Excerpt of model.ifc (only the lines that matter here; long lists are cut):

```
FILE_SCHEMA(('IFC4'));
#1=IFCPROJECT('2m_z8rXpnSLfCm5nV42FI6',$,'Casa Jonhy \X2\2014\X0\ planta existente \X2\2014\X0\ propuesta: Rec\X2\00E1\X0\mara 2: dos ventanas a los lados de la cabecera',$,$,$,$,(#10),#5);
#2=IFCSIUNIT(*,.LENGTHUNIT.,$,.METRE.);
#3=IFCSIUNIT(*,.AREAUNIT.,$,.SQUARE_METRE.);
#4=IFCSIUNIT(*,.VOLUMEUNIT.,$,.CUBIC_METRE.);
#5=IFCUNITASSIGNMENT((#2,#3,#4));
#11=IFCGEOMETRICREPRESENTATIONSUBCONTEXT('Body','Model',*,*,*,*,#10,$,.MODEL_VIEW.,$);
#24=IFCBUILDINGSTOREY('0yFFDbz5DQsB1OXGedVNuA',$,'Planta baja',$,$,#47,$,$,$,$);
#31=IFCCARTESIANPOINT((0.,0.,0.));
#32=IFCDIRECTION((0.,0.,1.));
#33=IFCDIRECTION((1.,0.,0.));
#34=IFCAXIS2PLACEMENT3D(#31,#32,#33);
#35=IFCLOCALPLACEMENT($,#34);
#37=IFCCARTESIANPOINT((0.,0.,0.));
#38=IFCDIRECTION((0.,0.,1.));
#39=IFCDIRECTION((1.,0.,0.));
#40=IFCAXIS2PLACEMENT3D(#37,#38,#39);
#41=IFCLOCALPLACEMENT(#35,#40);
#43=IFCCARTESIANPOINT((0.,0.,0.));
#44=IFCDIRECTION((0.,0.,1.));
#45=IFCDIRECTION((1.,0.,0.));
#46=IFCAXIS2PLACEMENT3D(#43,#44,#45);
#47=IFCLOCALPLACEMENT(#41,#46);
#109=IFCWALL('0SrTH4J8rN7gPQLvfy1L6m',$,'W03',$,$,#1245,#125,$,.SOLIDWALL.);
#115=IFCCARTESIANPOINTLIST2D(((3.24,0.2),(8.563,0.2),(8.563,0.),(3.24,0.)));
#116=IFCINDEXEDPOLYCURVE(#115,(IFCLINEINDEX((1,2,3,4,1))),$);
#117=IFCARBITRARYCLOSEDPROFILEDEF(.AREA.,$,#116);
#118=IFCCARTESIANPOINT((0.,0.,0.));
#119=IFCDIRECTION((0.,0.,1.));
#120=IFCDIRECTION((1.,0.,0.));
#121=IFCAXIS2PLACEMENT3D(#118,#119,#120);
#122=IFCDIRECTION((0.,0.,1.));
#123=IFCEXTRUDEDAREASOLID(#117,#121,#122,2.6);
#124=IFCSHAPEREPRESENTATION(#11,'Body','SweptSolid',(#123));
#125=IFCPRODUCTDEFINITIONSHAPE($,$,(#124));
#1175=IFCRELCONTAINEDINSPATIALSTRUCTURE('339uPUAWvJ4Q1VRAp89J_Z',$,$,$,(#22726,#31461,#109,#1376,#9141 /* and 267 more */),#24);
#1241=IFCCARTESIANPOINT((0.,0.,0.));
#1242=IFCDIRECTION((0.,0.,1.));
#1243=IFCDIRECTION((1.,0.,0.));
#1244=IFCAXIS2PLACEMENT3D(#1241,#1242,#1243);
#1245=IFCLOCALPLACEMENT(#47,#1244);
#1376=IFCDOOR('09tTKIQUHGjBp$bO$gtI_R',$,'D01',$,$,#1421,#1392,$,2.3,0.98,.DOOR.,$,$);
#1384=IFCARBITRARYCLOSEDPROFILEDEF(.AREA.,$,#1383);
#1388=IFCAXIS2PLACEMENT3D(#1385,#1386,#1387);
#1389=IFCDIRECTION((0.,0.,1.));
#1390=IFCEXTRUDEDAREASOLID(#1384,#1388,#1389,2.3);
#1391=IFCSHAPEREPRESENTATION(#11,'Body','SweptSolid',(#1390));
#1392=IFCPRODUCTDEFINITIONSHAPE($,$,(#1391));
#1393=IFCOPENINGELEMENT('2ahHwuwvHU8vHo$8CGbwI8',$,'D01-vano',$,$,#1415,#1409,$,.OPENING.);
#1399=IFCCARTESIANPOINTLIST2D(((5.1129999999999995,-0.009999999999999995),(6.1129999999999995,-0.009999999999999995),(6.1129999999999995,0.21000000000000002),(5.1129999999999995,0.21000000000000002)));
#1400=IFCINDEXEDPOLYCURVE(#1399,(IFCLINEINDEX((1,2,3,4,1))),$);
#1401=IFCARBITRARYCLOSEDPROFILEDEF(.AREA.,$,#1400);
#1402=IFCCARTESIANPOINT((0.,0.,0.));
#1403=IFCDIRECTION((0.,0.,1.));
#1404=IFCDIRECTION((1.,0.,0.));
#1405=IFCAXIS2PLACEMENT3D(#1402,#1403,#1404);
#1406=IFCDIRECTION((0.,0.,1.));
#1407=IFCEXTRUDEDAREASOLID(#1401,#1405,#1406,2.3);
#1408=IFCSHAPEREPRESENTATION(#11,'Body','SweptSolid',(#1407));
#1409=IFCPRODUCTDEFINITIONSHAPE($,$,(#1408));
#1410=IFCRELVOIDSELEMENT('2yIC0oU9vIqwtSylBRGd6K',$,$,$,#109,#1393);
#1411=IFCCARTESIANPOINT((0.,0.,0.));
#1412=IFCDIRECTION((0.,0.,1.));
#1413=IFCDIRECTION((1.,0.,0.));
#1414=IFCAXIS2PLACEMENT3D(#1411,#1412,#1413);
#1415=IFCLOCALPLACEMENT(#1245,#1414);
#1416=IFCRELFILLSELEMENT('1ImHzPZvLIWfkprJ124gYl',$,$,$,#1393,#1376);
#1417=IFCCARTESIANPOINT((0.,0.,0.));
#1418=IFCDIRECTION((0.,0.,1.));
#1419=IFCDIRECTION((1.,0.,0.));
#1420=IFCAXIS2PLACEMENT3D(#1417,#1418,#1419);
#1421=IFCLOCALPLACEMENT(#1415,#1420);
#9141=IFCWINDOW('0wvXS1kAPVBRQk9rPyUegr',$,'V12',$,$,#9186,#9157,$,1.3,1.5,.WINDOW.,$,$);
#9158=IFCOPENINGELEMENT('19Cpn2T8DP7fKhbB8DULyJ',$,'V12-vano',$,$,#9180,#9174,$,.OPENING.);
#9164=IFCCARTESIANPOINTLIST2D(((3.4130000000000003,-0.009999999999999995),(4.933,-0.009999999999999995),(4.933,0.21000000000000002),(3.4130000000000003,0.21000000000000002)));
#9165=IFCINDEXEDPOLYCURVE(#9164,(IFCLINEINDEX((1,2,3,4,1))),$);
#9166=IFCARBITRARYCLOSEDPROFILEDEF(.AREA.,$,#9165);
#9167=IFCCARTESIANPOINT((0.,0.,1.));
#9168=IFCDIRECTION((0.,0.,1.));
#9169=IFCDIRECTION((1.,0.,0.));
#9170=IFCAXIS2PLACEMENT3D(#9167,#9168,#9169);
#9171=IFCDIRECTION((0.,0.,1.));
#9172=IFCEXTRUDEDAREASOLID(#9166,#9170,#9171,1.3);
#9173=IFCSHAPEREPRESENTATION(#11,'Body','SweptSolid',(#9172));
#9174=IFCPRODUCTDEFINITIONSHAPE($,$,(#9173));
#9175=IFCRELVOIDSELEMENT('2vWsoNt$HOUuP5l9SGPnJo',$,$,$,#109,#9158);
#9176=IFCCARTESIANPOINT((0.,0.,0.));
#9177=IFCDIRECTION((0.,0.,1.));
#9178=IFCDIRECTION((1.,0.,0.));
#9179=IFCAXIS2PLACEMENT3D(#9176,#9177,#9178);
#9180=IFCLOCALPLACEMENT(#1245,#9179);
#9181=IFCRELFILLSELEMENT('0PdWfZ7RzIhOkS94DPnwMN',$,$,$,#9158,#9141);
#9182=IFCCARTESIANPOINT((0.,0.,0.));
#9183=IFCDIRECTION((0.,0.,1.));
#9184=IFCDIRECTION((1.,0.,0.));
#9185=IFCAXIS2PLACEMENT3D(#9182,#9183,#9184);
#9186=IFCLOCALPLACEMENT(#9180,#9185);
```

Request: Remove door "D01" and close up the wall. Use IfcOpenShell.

```python
import ifcopenshell
import ifcopenshell.api.feature
import ifcopenshell.api.root
import ifcopenshell.geom
import ifcopenshell.util.shape

model = ifcopenshell.open("model.ifc")
settings = ifcopenshell.geom.settings()


def volume(element):
    """Net volume in cubic metres, openings subtracted."""
    shape = ifcopenshell.geom.create_shape(settings, element)
    return ifcopenshell.util.shape.get_volume(shape.geometry)


door = model.by_id(1376)
opening = door.FillsVoids[0].RelatingOpeningElement
wall = opening.VoidsElements[0].RelatingBuildingElement
before = volume(wall)

ifcopenshell.api.root.remove_product(model, product=door)
ifcopenshell.api.feature.remove_feature(model, feature=opening)

after = volume(wall)

print(f"wall volume {before:.3f} -> {after:.3f} m3")

model.write("model_rev.ifc")
```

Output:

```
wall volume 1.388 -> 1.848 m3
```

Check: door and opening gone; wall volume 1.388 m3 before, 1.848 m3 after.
